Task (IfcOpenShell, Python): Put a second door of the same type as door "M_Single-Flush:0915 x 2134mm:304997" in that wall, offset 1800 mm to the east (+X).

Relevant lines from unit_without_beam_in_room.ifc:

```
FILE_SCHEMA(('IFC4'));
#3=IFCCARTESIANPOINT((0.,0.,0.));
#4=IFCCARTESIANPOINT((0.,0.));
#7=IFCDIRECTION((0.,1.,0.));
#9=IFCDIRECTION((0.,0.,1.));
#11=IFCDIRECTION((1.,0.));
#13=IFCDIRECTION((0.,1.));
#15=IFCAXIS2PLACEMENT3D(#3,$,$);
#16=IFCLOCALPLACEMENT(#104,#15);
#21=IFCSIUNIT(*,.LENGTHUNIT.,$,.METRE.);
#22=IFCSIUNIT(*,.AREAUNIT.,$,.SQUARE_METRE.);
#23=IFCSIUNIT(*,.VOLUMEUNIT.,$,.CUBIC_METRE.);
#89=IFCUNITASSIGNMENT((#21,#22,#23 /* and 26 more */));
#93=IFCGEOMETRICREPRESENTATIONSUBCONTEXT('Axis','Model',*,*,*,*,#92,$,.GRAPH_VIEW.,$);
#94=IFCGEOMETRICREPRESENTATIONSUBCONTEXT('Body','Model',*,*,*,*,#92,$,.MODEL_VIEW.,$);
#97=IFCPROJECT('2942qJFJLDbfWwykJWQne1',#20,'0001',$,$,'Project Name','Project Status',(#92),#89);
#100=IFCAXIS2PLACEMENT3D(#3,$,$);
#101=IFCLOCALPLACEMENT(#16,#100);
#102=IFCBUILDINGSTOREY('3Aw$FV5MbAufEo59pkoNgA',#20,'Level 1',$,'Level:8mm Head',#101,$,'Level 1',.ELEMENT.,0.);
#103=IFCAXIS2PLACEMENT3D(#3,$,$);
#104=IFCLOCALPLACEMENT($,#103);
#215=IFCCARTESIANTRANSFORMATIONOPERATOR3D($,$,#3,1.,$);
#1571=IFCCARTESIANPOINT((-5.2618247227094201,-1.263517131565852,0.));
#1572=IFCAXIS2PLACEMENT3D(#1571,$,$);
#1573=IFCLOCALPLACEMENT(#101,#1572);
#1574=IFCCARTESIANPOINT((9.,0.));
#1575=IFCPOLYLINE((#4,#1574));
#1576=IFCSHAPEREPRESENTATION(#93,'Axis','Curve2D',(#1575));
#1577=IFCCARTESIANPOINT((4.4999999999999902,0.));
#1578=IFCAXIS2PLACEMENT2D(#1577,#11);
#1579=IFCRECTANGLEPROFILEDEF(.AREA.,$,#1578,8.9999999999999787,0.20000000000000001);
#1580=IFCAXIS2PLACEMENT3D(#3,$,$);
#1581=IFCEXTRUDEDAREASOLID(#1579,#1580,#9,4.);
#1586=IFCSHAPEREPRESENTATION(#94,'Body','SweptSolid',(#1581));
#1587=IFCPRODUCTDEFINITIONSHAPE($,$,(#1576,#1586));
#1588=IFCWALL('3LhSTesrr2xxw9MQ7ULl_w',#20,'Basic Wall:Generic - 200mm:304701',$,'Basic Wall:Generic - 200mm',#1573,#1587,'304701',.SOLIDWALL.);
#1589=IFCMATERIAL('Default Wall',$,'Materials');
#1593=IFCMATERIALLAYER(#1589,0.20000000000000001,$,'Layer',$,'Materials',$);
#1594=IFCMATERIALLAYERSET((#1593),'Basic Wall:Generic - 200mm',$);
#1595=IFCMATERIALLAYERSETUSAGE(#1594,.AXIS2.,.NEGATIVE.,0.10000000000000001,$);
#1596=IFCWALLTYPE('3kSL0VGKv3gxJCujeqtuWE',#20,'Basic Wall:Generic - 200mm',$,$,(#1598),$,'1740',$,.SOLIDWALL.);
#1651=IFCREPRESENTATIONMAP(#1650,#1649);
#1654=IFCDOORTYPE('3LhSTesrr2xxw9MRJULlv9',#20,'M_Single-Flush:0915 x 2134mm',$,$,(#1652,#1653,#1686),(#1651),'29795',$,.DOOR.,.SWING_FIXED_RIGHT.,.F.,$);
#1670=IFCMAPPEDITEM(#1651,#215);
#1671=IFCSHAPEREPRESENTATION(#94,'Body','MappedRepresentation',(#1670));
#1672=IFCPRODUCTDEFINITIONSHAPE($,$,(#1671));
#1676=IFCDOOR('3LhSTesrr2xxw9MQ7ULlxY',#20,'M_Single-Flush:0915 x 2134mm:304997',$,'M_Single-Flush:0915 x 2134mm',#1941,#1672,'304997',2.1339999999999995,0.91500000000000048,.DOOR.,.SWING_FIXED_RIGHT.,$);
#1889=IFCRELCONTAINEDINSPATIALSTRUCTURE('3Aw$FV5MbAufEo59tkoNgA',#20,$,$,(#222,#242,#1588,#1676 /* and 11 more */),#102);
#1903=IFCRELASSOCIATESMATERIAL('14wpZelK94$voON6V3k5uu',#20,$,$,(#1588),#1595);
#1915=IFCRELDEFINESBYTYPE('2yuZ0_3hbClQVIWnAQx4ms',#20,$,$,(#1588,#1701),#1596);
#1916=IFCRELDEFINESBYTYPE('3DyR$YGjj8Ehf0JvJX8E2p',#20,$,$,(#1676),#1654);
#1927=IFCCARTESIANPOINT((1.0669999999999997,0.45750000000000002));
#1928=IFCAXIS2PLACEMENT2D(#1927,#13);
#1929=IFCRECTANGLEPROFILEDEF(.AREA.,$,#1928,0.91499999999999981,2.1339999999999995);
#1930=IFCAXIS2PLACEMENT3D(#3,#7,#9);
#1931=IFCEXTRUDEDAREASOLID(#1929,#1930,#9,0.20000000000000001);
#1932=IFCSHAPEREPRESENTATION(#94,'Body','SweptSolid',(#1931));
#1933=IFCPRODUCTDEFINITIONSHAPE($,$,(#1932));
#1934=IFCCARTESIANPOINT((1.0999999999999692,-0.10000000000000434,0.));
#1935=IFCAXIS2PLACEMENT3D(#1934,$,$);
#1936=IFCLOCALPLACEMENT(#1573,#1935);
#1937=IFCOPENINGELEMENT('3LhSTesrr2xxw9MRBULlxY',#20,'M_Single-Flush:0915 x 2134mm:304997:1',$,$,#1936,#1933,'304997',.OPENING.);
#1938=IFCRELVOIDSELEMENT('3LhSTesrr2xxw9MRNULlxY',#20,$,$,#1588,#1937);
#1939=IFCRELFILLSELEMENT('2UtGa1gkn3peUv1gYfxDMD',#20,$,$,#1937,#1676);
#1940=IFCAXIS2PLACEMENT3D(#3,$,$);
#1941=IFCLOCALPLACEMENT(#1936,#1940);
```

```python
import ifcopenshell
import ifcopenshell.api.feature
import ifcopenshell.api.geometry
import ifcopenshell.api.root
import ifcopenshell.geom
import ifcopenshell.util.element
import ifcopenshell.util.placement
import ifcopenshell.util.shape
import ifcopenshell.util.unit

model = ifcopenshell.open("unit_without_beam_in_room.ifc")
unit_scale = ifcopenshell.util.unit.calculate_unit_scale(model)
settings = ifcopenshell.geom.settings()


def volume(element):
    """Net volume in cubic metres, openings subtracted."""
    shape = ifcopenshell.geom.create_shape(settings, element)
    return ifcopenshell.util.shape.get_volume(shape.geometry)


def reuse_history(source, copy):
    """copy_class also copies each property set's owner history, people and application; keep the originals."""
    for rel in copy.IsDefinedBy:
        if rel.is_a("IfcRelDefinesByProperties") and (history := rel.RelatingPropertyDefinition.OwnerHistory):
            rel.RelatingPropertyDefinition.OwnerHistory = source.OwnerHistory
            ifcopenshell.util.element.remove_deep2(model, history)


door = model.by_id(1676)
opening = door.FillsVoids[0].RelatingOpeningElement
wall = opening.VoidsElements[0].RelatingBuildingElement
before = volume(wall)
shift = ifcopenshell.util.placement.get_local_placement(wall.ObjectPlacement)[:3, 0] * 1.8 / unit_scale

# copy_class copies the void relationship, type, container and properties, but no geometry.
new_opening = ifcopenshell.api.root.copy_class(model, product=opening)
new_opening.Representation = ifcopenshell.util.element.copy_deep(
    model, opening.Representation, exclude=["IfcGeometricRepresentationContext", "IfcRepresentationMap"]
)
new_opening.Name = "M_Single-Flush:0915 x 2134mm"
new_opening.Tag = None
new_door = ifcopenshell.api.root.copy_class(model, product=door)
new_door.Representation = ifcopenshell.util.element.copy_deep(
    model, door.Representation, exclude=["IfcGeometricRepresentationContext", "IfcRepresentationMap"]
)
new_door.Name = "M_Single-Flush:0915 x 2134mm"
new_door.Tag = None
reuse_history(door, new_door)
ifcopenshell.api.feature.add_filling(model, opening=new_opening, element=new_door)

for old, new in ((opening, new_opening), (door, new_door)):
    matrix = ifcopenshell.util.placement.get_local_placement(old.ObjectPlacement)
    matrix[:3, 3] += shift
    ifcopenshell.api.geometry.edit_object_placement(model, product=new, matrix=matrix, is_si=False)

after = volume(wall)

print(f"wall volume {before:.3f} -> {after:.3f} m3")

model.write("unit_without_beam_in_room_rev.ifc")
```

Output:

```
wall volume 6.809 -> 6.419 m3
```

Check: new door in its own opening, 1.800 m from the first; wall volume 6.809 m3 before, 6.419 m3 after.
